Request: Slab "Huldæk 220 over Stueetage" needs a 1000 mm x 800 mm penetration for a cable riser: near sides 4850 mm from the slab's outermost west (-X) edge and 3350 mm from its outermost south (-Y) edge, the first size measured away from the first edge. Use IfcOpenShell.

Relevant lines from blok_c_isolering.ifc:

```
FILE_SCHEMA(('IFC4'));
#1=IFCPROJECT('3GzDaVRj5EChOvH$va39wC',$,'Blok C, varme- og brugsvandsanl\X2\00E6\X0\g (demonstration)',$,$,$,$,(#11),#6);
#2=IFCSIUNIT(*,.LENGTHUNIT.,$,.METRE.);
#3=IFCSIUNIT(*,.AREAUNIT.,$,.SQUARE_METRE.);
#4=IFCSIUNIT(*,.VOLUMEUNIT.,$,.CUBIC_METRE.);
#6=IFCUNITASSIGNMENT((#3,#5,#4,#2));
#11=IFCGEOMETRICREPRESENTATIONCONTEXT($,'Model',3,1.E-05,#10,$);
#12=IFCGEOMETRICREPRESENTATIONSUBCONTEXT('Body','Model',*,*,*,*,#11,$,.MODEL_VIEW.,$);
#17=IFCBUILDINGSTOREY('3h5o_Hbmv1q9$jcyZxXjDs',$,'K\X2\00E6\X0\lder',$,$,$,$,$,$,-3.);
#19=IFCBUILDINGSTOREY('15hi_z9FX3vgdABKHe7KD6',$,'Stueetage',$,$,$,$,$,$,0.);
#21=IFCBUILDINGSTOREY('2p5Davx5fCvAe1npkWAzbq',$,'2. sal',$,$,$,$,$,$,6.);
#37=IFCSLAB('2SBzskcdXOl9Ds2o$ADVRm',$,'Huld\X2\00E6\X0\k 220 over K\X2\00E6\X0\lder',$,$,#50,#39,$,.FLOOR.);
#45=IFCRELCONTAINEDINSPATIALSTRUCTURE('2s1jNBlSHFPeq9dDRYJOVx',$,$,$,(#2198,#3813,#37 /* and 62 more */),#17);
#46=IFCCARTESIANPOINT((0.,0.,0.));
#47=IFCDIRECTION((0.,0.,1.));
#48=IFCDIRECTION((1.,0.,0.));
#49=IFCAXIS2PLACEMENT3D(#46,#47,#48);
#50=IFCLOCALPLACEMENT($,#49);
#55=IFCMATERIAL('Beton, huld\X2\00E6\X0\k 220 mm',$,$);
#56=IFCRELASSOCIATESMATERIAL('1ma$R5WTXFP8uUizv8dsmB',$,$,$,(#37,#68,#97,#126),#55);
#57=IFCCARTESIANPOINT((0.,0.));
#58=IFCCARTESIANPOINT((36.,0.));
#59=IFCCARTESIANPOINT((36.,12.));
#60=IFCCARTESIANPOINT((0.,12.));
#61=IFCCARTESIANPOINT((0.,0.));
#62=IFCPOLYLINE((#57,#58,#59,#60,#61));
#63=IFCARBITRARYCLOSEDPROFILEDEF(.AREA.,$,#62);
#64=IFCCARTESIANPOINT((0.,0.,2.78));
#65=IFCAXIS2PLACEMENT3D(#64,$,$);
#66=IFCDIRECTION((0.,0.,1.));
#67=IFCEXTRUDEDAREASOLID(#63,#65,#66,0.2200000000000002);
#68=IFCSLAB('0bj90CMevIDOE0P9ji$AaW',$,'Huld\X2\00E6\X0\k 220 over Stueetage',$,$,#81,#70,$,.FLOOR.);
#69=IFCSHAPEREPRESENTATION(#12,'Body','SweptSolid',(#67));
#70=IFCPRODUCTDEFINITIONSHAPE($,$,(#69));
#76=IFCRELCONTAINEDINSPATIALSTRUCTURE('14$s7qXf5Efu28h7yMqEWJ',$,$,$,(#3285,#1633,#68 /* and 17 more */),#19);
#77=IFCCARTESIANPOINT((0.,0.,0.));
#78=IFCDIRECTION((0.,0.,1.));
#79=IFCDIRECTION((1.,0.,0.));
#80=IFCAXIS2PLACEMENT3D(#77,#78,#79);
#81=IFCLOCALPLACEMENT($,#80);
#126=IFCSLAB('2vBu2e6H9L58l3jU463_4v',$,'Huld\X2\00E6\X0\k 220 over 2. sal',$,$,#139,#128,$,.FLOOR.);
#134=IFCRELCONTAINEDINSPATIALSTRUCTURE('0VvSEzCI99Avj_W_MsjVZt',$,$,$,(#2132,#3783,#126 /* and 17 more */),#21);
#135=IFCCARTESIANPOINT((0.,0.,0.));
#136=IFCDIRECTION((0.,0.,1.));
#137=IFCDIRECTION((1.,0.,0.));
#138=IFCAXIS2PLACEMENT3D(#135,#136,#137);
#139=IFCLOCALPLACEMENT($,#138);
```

```python
import numpy as np
import ifcopenshell
import ifcopenshell.api.feature
import ifcopenshell.api.geometry
import ifcopenshell.api.root
import ifcopenshell.geom
import ifcopenshell.util.placement
import ifcopenshell.util.representation
import ifcopenshell.util.shape
import ifcopenshell.util.unit

model = ifcopenshell.open("blok_c_isolering.ifc")
unit_scale = ifcopenshell.util.unit.calculate_unit_scale(model)
settings = ifcopenshell.geom.settings()


def volume(element):
    """Net volume in cubic metres, openings subtracted."""
    shape = ifcopenshell.geom.create_shape(settings, element)
    return ifcopenshell.util.shape.get_volume(shape.geometry)


slab = model.by_guid("0bj90CMevIDOE0P9ji$AaW")
before = volume(slab)

# Extent in the slab's own axes, in metres. The edges named are its -X and -Y sides.
slab_shape = ifcopenshell.geom.create_shape(settings, slab)
vertices = ifcopenshell.util.shape.get_vertices(slab_shape.geometry)
x_min, y_min, bottom = vertices.min(axis=0)
top = vertices[:, 2].max()

opening = ifcopenshell.api.root.create_entity(model, ifc_class="IfcOpeningElement", name="Cable riser opening", predefined_type="OPENING")
context = ifcopenshell.util.representation.get_context(model, "Model", "Body", "MODEL_VIEW")
width, depth = 1, 0.8
outline = [(0.0, 0.0), (width, 0.0), (width, depth), (0.0, depth), (0.0, 0.0)]
# Overshoot both faces by 50 mm so the cut is clean.
shape = ifcopenshell.api.geometry.add_slab_representation(
    model, context=context, depth=top - bottom + 0.1, polyline=outline
)
ifcopenshell.api.geometry.assign_representation(model, product=opening, representation=shape)

matrix = ifcopenshell.util.placement.get_local_placement(slab.ObjectPlacement)
matrix[:, 3] = matrix @ np.append(np.array([x_min + 4.85, y_min + 3.35, bottom - 0.05]) / unit_scale, 1.0)
ifcopenshell.api.geometry.edit_object_placement(model, product=opening, matrix=matrix, is_si=False)
ifcopenshell.api.feature.add_feature(model, feature=opening, element=slab)

after = volume(slab)

print(f"slab volume {before:.3f} -> {after:.3f} m3")

model.write("blok_c_isolering_updated.ifc")
```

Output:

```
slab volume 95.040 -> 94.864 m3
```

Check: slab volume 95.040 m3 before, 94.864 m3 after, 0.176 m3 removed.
